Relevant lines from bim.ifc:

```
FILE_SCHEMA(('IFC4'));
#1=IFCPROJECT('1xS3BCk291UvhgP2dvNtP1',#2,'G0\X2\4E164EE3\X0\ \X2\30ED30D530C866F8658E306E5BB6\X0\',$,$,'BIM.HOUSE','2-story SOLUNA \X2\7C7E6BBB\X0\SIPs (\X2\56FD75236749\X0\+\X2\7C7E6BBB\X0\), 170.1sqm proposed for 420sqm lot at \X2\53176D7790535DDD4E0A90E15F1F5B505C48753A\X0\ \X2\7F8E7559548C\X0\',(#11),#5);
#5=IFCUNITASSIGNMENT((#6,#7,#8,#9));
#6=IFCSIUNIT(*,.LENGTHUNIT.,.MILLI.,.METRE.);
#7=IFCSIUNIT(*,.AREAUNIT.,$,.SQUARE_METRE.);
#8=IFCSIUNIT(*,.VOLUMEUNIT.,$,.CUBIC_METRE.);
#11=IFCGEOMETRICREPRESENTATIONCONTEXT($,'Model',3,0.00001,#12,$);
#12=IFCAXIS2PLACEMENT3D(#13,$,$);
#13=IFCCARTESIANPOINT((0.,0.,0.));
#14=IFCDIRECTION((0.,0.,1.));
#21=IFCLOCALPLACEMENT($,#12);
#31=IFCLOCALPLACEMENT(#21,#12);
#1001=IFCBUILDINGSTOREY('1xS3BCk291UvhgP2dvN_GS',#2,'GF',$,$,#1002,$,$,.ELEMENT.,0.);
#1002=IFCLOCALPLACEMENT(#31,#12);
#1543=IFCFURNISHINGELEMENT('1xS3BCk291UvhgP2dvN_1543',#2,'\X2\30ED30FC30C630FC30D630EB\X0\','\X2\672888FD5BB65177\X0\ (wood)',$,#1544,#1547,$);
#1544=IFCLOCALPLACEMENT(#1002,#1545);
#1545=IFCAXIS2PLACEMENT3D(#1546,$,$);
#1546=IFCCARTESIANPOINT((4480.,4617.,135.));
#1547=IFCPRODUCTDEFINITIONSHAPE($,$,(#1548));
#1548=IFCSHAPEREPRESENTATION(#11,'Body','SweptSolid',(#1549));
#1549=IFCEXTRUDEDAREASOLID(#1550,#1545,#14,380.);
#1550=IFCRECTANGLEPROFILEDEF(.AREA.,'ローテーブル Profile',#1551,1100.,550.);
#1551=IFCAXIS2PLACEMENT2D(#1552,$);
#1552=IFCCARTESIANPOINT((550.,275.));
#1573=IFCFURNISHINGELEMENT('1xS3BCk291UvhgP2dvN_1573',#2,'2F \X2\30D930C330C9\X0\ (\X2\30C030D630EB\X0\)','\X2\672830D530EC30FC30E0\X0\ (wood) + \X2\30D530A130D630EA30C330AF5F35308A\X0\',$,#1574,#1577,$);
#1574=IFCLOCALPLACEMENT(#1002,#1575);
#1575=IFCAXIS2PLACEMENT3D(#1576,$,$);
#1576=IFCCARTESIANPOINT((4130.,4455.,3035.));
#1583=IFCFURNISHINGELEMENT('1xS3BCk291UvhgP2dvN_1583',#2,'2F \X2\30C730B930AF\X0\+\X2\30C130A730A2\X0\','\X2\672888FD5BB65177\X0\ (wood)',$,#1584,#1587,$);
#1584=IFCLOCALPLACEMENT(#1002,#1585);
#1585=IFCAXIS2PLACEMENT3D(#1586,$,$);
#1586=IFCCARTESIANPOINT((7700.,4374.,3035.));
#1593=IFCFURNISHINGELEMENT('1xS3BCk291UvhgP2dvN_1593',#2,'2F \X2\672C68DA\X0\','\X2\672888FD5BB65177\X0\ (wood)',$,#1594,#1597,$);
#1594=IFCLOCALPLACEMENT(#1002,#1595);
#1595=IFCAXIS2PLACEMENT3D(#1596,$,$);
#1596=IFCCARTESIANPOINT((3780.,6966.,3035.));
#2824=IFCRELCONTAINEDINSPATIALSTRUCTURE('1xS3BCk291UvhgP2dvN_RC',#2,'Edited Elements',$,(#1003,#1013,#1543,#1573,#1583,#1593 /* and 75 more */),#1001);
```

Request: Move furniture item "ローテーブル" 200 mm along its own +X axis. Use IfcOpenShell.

```python
import ifcopenshell
import ifcopenshell.api.geometry
import ifcopenshell.util.placement
import ifcopenshell.util.unit

model = ifcopenshell.open("bim.ifc")
unit_scale = ifcopenshell.util.unit.calculate_unit_scale(model)

item = model.by_guid("1xS3BCk291UvhgP2dvN_1543")
matrix = ifcopenshell.util.placement.get_local_placement(item.ObjectPlacement)
matrix[:3, 3] += matrix[:3, 0] * 0.2 / unit_scale
ifcopenshell.api.geometry.edit_object_placement(model, product=item, matrix=matrix, is_si=False)

print(ifcopenshell.util.placement.get_local_placement(item.ObjectPlacement).round(3) + 0.0)

model.write("bim_edited.ifc")
```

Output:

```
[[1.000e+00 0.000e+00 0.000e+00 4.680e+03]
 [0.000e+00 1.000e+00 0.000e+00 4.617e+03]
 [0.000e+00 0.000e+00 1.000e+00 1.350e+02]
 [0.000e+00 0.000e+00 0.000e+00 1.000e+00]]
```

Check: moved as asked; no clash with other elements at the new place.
